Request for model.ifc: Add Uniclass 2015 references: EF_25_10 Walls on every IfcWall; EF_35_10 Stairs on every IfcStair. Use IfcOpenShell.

First a look at what the model holds.

```python
import ifcopenshell

model = ifcopenshell.open("model.ifc")
print(model.schema)
print("classifications:", [c.Name for c in model.by_type("IfcClassification")])
for ifc_class in ("IfcDoor", "IfcRoof", "IfcStair", "IfcWall", "IfcWindow"):
    print(ifc_class, len(model.by_type(ifc_class)))
```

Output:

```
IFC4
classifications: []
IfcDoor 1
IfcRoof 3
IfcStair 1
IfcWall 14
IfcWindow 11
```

```python
import ifcopenshell
import ifcopenshell.api.classification

model = ifcopenshell.open("model.ifc")

system = ifcopenshell.api.classification.add_classification(model, classification="Uniclass 2015")

codes = {
    "IfcWall": ("EF_25_10", "Walls"),
    "IfcStair": ("EF_35_10", "Stairs"),
}
for ifc_class, (code, name) in codes.items():
    products = model.by_type(ifc_class)
    ifcopenshell.api.classification.add_reference(
        model, products=products, classification=system, identification=code, name=name
    )
    print(code, len(products))

model.write("model_updated.ifc")
```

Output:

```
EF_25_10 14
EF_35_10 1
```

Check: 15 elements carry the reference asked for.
